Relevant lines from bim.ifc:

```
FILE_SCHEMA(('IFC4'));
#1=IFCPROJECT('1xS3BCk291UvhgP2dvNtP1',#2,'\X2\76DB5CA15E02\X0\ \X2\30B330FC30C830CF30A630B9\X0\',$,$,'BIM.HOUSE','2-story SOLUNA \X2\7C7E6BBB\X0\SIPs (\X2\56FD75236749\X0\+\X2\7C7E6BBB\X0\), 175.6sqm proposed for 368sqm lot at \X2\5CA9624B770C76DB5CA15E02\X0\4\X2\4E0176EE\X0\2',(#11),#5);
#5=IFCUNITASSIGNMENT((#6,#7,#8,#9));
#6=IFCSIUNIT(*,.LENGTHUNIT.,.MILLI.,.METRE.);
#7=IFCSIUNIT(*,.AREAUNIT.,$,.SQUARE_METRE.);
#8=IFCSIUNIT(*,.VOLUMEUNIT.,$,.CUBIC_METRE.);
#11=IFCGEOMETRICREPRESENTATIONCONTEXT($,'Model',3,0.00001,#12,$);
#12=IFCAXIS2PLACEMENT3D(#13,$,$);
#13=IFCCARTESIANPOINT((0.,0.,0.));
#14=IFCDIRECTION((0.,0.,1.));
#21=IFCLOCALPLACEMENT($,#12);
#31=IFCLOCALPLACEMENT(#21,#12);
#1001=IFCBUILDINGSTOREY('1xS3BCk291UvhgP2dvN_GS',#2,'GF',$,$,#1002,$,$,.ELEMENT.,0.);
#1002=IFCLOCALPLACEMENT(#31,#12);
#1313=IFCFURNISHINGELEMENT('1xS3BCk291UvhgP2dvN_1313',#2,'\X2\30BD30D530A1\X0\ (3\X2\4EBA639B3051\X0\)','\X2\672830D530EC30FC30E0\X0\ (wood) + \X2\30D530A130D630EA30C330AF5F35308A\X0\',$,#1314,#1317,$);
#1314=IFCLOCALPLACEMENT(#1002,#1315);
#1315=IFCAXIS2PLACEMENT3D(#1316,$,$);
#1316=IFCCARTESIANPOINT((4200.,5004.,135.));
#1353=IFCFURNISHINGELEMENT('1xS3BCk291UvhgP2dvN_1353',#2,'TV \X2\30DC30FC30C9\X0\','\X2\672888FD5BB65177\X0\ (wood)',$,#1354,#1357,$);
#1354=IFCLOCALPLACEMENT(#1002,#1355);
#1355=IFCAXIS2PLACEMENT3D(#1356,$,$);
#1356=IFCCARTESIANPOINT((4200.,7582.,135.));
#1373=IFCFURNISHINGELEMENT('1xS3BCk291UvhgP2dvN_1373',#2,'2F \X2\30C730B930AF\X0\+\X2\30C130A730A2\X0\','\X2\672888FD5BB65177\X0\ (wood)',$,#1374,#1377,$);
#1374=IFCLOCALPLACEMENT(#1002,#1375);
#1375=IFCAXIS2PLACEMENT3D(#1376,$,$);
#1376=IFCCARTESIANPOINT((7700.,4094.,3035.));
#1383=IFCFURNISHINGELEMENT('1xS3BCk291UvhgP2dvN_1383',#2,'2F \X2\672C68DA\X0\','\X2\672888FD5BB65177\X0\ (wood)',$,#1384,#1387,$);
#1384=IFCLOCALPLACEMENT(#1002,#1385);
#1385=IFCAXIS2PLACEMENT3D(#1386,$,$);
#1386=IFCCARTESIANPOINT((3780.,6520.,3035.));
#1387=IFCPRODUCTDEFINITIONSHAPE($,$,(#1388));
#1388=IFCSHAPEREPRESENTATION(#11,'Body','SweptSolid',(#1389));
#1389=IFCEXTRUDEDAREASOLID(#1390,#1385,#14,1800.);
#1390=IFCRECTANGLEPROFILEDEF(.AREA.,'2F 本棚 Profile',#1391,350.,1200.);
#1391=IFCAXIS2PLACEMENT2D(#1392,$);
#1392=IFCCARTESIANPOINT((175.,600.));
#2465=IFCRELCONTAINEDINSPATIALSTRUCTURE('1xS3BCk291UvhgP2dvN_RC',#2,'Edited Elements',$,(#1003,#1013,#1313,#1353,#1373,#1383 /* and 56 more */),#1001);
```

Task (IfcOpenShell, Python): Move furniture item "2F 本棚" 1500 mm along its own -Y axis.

```python
import ifcopenshell
import ifcopenshell.api.geometry
import ifcopenshell.util.placement
import ifcopenshell.util.unit

model = ifcopenshell.open("bim.ifc")
unit_scale = ifcopenshell.util.unit.calculate_unit_scale(model)

item = model.by_guid("1xS3BCk291UvhgP2dvN_1383")
matrix = ifcopenshell.util.placement.get_local_placement(item.ObjectPlacement)
matrix[:3, 3] -= matrix[:3, 1] * 1.5 / unit_scale
ifcopenshell.api.geometry.edit_object_placement(model, product=item, matrix=matrix, is_si=False)

print(ifcopenshell.util.placement.get_local_placement(item.ObjectPlacement).round(3) + 0.0)

model.write("bim_updated.ifc")
```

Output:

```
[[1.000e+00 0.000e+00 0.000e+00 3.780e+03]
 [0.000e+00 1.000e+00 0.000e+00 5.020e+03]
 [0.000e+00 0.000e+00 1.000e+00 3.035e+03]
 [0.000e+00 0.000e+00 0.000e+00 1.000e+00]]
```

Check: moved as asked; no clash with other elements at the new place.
